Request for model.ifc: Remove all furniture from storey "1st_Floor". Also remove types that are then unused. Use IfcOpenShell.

First a look at what the model holds.

```python
import ifcopenshell
import ifcopenshell.util.element

model = ifcopenshell.open("model.ifc")
print(model.schema)
storey = next(s for s in model.by_type("IfcBuildingStorey") if s.Name == "1st_Floor")
furniture = [e for e in ifcopenshell.util.element.get_decomposition(storey) if e.is_a("IfcFurnishingElement")]
seen = {}
for e in furniture:
    element_type = ifcopenshell.util.element.get_type(e)
    name = element_type.Name if element_type not in (None, e) else None
    seen[name] = seen.get(name, 0) + 1
for name, count in sorted(seen.items(), key=str):
    print(count, "x", name)
```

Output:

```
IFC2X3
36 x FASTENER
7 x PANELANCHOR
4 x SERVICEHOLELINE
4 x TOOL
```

```python
import ifcopenshell
import ifcopenshell.api.root
import ifcopenshell.util.element

model = ifcopenshell.open("model.ifc")

storey = next(s for s in model.by_type("IfcBuildingStorey") if s.Name == "1st_Floor")
furniture = [e for e in ifcopenshell.util.element.get_decomposition(storey) if e.is_a("IfcFurnishingElement")]
types = {ifcopenshell.util.element.get_type(e) for e in furniture} - {None, *furniture}

for e in furniture:
    ifcopenshell.api.root.remove_product(model, product=e)
print(len(furniture), "removed")

unused = [t for t in types if not ifcopenshell.util.element.get_types(t)]
for t in unused:
    ifcopenshell.api.root.remove_product(model, product=t)
print(len(unused), "unused types removed")

model.write("model_edited.ifc")
```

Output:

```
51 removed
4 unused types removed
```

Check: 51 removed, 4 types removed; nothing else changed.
